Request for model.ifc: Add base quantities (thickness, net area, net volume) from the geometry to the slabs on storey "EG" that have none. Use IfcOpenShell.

First a look at what the model holds.

```python
import ifcopenshell
import ifcopenshell.util.element
import ifcopenshell.util.unit

model = ifcopenshell.open("model.ifc")
print(model.schema)
for unit_type in ("LENGTHUNIT", "AREAUNIT", "VOLUMEUNIT"):
    print(unit_type, ifcopenshell.util.unit.calculate_unit_scale(model, unit_type))
storey = next(s for s in model.by_type("IfcBuildingStorey") if s.Name == "EG")
slabs = [e for e in ifcopenshell.util.element.get_decomposition(storey) if e.is_a("IfcSlab")]
for e in sorted(slabs, key=lambda e: e.id()):
    print(e.id(), e.is_a(), e.Name, list(ifcopenshell.util.element.get_psets(e, qtos_only=True)), sep=" | ")
```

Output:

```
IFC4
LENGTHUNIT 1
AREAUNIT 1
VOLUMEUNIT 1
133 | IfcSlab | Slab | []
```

```python
import ifcopenshell
import ifcopenshell.api.pset
import ifcopenshell.geom
import ifcopenshell.util.element
import ifcopenshell.util.shape
import ifcopenshell.util.unit

model = ifcopenshell.open("model.ifc")
unit_scale = ifcopenshell.util.unit.calculate_unit_scale(model)
area_scale = ifcopenshell.util.unit.calculate_unit_scale(model, "AREAUNIT")
volume_scale = ifcopenshell.util.unit.calculate_unit_scale(model, "VOLUMEUNIT")
settings = ifcopenshell.geom.settings()

storey = next(s for s in model.by_type("IfcBuildingStorey") if s.Name == "EG")
slabs = [e for e in ifcopenshell.util.element.get_decomposition(storey) if e.is_a("IfcSlab")]

for e in sorted(slabs, key=lambda e: e.id()):
    if ifcopenshell.util.element.get_psets(e, qtos_only=True, should_inherit=False):
        continue
    # Geometry comes back in metres, in the element's own axes.
    shape = ifcopenshell.geom.create_shape(settings, e)
    values = {
        "Width": ifcopenshell.util.shape.get_z(shape.geometry) / unit_scale,
        "NetArea": ifcopenshell.util.shape.get_footprint_area(shape.geometry) / area_scale,
        "NetVolume": ifcopenshell.util.shape.get_volume(shape.geometry) / volume_scale,
    }
    qto = ifcopenshell.api.pset.add_qto(model, product=e, name="Qto_SlabBaseQuantities")
    ifcopenshell.api.pset.edit_qto(model, qto=qto, properties=values)
    print(e.id(), {k: round(v, 3) for k, v in values.items()})

model.write("model_rev.ifc")
```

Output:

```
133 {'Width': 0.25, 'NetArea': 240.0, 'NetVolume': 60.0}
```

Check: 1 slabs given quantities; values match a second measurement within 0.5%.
